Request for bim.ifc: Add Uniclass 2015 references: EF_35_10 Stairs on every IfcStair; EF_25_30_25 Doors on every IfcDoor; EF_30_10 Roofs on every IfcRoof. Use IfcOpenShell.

First a look at what the model holds.

```python
import ifcopenshell

model = ifcopenshell.open("bim.ifc")
print(model.schema)
print("classifications:", [c.Name for c in model.by_type("IfcClassification")])
for ifc_class in ("IfcDoor", "IfcRoof", "IfcStair", "IfcWall", "IfcWindow"):
    print(ifc_class, len(model.by_type(ifc_class)))
```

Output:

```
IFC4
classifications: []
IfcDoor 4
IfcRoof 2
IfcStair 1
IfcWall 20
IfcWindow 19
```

```python
import ifcopenshell
import ifcopenshell.api.classification

model = ifcopenshell.open("bim.ifc")

system = ifcopenshell.api.classification.add_classification(model, classification="Uniclass 2015")

codes = {
    "IfcStair": ("EF_35_10", "Stairs"),
    "IfcDoor": ("EF_25_30_25", "Doors"),
    "IfcRoof": ("EF_30_10", "Roofs"),
}
for ifc_class, (code, name) in codes.items():
    products = model.by_type(ifc_class)
    ifcopenshell.api.classification.add_reference(
        model, products=products, classification=system, identification=code, name=name
    )
    print(code, len(products))

model.write("bim_rev.ifc")
```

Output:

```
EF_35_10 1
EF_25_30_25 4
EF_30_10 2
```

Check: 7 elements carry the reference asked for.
